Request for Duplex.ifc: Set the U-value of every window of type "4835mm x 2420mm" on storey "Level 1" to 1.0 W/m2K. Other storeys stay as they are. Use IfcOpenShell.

First a look at what the model holds.

```python
import ifcopenshell
import ifcopenshell.util.element

model = ifcopenshell.open("Duplex.ifc")
print(model.schema)
storey = next(s for s in model.by_type("IfcBuildingStorey") if s.Name == "Level 1")
windows = [e for e in ifcopenshell.util.element.get_decomposition(storey) if e.is_a("IfcWindow")]
seen = {}
for e in windows:
    element_type = ifcopenshell.util.element.get_type(e)
    key = (element_type.Name if element_type != e and element_type else None, ifcopenshell.util.element.get_pset(e, "Pset_WindowCommon", "ThermalTransmittance"))
    seen[key] = seen.get(key, 0) + 1
for (name, value), count in sorted(seen.items(), key=str):
    print(count, "x", name, "|", value)
```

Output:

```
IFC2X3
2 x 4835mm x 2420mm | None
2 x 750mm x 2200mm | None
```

```python
import ifcopenshell
import ifcopenshell.api.pset
import ifcopenshell.util.element

model = ifcopenshell.open("Duplex.ifc")

storey = next(s for s in model.by_type("IfcBuildingStorey") if s.Name == "Level 1")
windows = [e for e in ifcopenshell.util.element.get_decomposition(storey) if e.is_a("IfcWindow")]

count = 0
for e in windows:
    element_type = ifcopenshell.util.element.get_type(e)
    if element_type in (None, e) or element_type.Name != "4835mm x 2420mm":
        continue
    # add_pset returns the element's existing set when there is one.
    pset = ifcopenshell.api.pset.add_pset(model, product=e, name="Pset_WindowCommon")
    ifcopenshell.api.pset.edit_pset(model, pset=pset, properties={"ThermalTransmittance": 1.0})
    count += 1

print(count, "windows updated")

model.write("Duplex-out.ifc")
```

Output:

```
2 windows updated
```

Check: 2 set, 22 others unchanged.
